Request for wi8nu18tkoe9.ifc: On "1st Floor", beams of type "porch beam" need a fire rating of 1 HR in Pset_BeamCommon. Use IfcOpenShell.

First a look at what the model holds.

```python
import ifcopenshell
import ifcopenshell.util.element

model = ifcopenshell.open("wi8nu18tkoe9.ifc")
print(model.schema)
storey = next(s for s in model.by_type("IfcBuildingStorey") if s.Name == "1st Floor")
beams = [e for e in ifcopenshell.util.element.get_decomposition(storey) if e.is_a("IfcBeam")]
seen = {}
for e in beams:
    element_type = ifcopenshell.util.element.get_type(e)
    key = (element_type.Name if element_type != e and element_type else None, ifcopenshell.util.element.get_pset(e, "Pset_BeamCommon", "FireRating"))
    seen[key] = seen.get(key, 0) + 1
for (name, value), count in sorted(seen.items(), key=str):
    print(count, "x", name, "|", value)
```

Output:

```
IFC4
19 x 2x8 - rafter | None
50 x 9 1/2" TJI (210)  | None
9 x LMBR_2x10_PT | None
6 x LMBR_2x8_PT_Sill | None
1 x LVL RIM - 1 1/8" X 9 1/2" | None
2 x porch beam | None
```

```python
import ifcopenshell
import ifcopenshell.api.pset
import ifcopenshell.util.element

model = ifcopenshell.open("wi8nu18tkoe9.ifc")

storey = next(s for s in model.by_type("IfcBuildingStorey") if s.Name == "1st Floor")
beams = [e for e in ifcopenshell.util.element.get_decomposition(storey) if e.is_a("IfcBeam")]

count = 0
for e in beams:
    element_type = ifcopenshell.util.element.get_type(e)
    if element_type in (None, e) or element_type.Name != "porch beam":
        continue
    # add_pset returns the element's existing set when there is one.
    pset = ifcopenshell.api.pset.add_pset(model, product=e, name="Pset_BeamCommon")
    ifcopenshell.api.pset.edit_pset(model, pset=pset, properties={"FireRating": "1 HR"})
    count += 1

print(count, "beams updated")

model.write("wi8nu18tkoe9_v2.ifc")
```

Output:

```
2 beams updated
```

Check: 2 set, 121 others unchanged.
